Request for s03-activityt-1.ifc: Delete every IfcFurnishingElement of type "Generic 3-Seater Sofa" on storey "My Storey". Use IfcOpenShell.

First a look at what the model holds.

```python
import ifcopenshell
import ifcopenshell.util.element

model = ifcopenshell.open("s03-activityt-1.ifc")
print(model.schema)
storey = next(s for s in model.by_type("IfcBuildingStorey") if s.Name == "My Storey")
furniture = [e for e in ifcopenshell.util.element.get_decomposition(storey) if e.is_a("IfcFurnishingElement")]
seen = {}
for e in furniture:
    element_type = ifcopenshell.util.element.get_type(e)
    name = element_type.Name if element_type not in (None, e) else None
    seen[name] = seen.get(name, 0) + 1
for name, count in sorted(seen.items(), key=str):
    print(count, "x", name)
```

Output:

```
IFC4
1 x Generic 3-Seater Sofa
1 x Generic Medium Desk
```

```python
import ifcopenshell
import ifcopenshell.api.root
import ifcopenshell.util.element

model = ifcopenshell.open("s03-activityt-1.ifc")

storey = next(s for s in model.by_type("IfcBuildingStorey") if s.Name == "My Storey")
furniture = [e for e in ifcopenshell.util.element.get_decomposition(storey) if e.is_a("IfcFurnishingElement")]
targets = [e for e in furniture if (t := ifcopenshell.util.element.get_type(e)) not in (None, e) and t.Name == "Generic 3-Seater Sofa"]

for e in targets:
    ifcopenshell.api.root.remove_product(model, product=e)
print(len(targets), "removed")

model.write("s03-activityt-1_rev.ifc")
```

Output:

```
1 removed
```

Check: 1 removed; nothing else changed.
